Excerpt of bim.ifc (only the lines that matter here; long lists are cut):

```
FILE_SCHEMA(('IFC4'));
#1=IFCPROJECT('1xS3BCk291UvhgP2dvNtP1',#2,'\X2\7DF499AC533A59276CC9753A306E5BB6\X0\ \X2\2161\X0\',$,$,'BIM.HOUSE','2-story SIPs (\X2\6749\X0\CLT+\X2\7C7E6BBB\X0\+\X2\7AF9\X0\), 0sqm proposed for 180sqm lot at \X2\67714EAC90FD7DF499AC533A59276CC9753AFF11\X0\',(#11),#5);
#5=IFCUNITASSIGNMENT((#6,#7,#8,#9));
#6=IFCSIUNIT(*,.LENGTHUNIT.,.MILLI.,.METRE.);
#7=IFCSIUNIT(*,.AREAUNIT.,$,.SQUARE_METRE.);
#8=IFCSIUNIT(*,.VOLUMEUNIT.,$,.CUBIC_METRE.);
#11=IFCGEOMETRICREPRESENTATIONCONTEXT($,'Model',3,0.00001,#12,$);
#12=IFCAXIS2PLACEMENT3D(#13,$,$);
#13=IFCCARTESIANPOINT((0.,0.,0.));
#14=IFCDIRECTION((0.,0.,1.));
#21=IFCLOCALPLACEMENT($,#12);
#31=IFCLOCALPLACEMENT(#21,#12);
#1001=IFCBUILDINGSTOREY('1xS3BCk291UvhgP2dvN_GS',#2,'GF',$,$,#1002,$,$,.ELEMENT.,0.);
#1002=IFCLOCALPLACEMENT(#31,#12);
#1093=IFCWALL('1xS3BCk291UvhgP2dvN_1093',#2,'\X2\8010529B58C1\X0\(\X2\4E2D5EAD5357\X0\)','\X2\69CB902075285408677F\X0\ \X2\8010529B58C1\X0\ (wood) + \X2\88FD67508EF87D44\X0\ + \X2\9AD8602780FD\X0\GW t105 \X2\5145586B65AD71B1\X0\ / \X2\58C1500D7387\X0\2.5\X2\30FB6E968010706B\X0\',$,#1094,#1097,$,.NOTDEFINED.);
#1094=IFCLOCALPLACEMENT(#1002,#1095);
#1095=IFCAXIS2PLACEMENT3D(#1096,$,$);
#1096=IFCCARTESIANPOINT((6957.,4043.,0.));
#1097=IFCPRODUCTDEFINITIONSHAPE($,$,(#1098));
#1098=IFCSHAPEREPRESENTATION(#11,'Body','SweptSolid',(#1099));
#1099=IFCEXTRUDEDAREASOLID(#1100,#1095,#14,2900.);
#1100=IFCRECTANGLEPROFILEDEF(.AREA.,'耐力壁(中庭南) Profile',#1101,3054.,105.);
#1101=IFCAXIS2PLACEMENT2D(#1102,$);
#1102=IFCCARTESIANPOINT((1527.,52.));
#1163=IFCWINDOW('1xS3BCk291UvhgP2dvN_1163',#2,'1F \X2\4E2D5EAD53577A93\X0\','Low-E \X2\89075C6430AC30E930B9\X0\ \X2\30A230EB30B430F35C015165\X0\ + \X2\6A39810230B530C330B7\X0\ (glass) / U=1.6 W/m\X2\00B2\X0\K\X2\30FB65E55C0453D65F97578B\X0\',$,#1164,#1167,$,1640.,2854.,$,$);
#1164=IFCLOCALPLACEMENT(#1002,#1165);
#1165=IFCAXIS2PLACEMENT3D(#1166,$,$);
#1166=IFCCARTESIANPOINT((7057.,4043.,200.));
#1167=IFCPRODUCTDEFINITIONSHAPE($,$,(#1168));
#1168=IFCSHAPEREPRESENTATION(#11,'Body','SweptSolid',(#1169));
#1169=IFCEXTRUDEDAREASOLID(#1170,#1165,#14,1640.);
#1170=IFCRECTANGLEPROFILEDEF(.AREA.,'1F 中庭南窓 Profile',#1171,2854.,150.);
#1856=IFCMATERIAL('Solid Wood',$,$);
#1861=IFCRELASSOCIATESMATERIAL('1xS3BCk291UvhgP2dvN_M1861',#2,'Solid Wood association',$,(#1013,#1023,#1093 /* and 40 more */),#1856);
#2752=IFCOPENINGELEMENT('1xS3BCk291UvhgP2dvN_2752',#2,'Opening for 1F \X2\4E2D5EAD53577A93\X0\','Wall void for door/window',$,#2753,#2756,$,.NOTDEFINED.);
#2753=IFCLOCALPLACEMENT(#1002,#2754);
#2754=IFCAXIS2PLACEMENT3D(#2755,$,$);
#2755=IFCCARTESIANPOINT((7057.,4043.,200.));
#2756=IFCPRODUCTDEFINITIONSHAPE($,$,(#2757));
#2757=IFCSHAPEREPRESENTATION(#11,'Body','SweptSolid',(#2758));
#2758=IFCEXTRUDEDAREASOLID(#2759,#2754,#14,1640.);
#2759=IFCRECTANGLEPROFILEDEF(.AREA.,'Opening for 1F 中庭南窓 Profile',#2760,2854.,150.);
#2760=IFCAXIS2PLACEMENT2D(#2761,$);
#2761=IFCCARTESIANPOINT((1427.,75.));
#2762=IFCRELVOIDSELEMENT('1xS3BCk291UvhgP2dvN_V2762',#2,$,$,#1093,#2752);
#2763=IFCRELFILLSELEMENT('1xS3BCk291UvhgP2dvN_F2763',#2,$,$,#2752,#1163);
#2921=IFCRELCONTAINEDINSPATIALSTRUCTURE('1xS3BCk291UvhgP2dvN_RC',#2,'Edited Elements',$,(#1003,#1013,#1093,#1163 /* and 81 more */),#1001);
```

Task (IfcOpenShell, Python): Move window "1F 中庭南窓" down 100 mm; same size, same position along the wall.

```python
import numpy as np
import ifcopenshell
import ifcopenshell.api.geometry
import ifcopenshell.util.placement
import ifcopenshell.util.unit

model = ifcopenshell.open("bim.ifc")
unit_scale = ifcopenshell.util.unit.calculate_unit_scale(model)

window = model.by_guid("1xS3BCk291UvhgP2dvN_1163")
opening = window.FillsVoids[0].RelatingOpeningElement
dz = -100.0

shift = np.array([0.0, 0.0, dz])
# The window is not placed relative to its opening, so move both.
for product in (opening, window):
    matrix = ifcopenshell.util.placement.get_local_placement(product.ObjectPlacement)
    matrix[:3, 3] += shift
    ifcopenshell.api.geometry.edit_object_placement(model, product=product, matrix=matrix, is_si=False)

print(f"moved by {dz * unit_scale:+.3f} m")

model.write("bim_rev.ifc")
```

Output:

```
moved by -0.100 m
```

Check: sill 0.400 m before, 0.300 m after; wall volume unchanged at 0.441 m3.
